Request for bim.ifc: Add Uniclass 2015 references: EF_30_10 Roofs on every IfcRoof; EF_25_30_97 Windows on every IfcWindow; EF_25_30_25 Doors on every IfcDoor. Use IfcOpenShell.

First a look at what the model holds.

```python
import ifcopenshell

model = ifcopenshell.open("bim.ifc")
print(model.schema)
print("classifications:", [c.Name for c in model.by_type("IfcClassification")])
for ifc_class in ("IfcDoor", "IfcRoof", "IfcStair", "IfcWall", "IfcWindow"):
    print(ifc_class, len(model.by_type(ifc_class)))
```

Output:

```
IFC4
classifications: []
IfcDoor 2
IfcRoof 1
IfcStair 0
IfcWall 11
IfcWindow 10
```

```python
import ifcopenshell
import ifcopenshell.api.classification

model = ifcopenshell.open("bim.ifc")

system = ifcopenshell.api.classification.add_classification(model, classification="Uniclass 2015")

codes = {
    "IfcRoof": ("EF_30_10", "Roofs"),
    "IfcWindow": ("EF_25_30_97", "Windows"),
    "IfcDoor": ("EF_25_30_25", "Doors"),
}
for ifc_class, (code, name) in codes.items():
    products = model.by_type(ifc_class)
    ifcopenshell.api.classification.add_reference(
        model, products=products, classification=system, identification=code, name=name
    )
    print(code, len(products))

model.write("bim_rev.ifc")
```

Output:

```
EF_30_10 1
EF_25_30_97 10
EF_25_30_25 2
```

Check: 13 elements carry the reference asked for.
